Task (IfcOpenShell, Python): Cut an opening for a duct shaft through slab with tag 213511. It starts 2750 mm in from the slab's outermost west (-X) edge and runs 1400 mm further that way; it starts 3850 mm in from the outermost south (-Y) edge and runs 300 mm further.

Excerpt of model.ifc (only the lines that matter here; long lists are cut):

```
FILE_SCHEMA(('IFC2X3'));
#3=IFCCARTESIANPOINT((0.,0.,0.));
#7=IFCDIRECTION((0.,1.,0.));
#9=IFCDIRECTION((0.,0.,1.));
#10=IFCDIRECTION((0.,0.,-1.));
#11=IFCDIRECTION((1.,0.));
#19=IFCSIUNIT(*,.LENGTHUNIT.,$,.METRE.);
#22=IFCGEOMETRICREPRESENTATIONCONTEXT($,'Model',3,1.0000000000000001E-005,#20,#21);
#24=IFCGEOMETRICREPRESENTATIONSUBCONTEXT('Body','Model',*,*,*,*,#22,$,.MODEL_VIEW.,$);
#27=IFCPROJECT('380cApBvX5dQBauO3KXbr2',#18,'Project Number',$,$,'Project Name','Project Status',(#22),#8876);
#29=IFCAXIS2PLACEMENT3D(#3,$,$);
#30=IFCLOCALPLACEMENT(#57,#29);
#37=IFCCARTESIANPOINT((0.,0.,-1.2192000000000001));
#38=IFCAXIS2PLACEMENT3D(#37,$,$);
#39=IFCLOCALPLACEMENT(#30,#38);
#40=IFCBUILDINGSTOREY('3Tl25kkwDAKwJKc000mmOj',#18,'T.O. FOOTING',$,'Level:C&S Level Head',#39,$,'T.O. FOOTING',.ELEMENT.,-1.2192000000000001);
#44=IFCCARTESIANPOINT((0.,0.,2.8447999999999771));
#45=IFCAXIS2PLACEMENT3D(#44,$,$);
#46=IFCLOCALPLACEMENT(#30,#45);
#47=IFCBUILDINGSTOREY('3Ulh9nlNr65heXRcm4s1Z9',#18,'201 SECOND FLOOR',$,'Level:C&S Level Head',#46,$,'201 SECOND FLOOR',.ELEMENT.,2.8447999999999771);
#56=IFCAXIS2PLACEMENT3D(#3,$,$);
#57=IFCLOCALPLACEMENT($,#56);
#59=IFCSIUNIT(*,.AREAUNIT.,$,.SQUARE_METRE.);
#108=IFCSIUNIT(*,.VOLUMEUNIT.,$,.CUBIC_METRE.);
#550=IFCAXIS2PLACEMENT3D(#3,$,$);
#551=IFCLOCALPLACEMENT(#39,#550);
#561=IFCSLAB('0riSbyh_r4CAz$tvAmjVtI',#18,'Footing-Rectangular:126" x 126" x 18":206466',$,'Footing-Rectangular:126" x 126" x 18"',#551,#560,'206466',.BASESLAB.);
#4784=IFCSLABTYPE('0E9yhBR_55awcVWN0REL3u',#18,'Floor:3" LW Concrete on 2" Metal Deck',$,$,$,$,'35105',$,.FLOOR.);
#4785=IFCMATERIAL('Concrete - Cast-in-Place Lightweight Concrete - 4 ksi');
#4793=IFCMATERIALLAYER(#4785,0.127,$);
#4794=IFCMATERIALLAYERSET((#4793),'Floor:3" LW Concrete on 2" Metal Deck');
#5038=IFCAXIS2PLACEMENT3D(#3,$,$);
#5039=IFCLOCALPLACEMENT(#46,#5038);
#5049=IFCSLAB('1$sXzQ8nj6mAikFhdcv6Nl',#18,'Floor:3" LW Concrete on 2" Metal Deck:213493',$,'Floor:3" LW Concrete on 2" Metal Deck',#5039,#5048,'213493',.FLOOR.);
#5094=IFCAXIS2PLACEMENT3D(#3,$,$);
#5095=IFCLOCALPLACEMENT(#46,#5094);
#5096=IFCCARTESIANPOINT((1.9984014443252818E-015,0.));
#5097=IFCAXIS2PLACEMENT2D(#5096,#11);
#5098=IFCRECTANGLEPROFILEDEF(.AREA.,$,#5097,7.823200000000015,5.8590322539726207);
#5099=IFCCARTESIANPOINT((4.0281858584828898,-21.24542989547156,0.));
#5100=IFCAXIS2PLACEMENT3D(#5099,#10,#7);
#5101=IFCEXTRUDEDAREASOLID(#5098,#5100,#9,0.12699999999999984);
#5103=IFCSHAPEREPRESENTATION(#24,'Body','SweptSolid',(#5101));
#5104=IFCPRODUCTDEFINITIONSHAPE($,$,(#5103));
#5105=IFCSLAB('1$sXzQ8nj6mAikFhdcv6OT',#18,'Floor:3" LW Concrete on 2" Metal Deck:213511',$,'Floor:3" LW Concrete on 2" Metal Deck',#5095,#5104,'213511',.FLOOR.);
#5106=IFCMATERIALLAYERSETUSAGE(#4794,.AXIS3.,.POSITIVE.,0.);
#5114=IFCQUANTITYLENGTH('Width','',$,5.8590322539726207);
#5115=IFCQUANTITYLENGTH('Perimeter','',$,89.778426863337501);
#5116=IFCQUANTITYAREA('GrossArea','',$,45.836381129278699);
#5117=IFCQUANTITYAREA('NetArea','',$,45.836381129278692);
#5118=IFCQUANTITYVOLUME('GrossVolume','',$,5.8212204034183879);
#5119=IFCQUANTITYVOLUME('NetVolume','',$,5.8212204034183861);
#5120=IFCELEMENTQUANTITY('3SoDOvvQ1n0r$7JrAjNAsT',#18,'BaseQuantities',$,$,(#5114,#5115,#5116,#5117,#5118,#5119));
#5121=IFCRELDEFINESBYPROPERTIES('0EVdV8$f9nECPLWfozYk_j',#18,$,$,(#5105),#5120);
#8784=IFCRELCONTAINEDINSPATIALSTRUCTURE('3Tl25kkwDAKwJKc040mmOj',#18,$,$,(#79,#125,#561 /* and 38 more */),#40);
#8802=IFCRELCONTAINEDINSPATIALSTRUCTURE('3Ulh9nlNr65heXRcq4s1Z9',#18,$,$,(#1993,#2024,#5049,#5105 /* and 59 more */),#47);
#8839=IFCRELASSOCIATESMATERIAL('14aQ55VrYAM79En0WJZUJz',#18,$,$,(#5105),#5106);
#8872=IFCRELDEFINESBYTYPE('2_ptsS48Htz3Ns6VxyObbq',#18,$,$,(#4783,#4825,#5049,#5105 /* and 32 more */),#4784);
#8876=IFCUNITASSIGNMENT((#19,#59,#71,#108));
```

```python
import numpy as np
import ifcopenshell
import ifcopenshell.api.feature
import ifcopenshell.api.geometry
import ifcopenshell.api.pset
import ifcopenshell.api.root
import ifcopenshell.geom
import ifcopenshell.util.element
import ifcopenshell.util.placement
import ifcopenshell.util.representation
import ifcopenshell.util.shape
import ifcopenshell.util.unit

model = ifcopenshell.open("model.ifc")
unit_scale = ifcopenshell.util.unit.calculate_unit_scale(model)
area_scale = ifcopenshell.util.unit.calculate_unit_scale(model, "AREAUNIT")
volume_scale = ifcopenshell.util.unit.calculate_unit_scale(model, "VOLUMEUNIT")
settings = ifcopenshell.geom.settings()


def volume(element):
    """Net volume in cubic metres, openings subtracted."""
    shape = ifcopenshell.geom.create_shape(settings, element)
    return ifcopenshell.util.shape.get_volume(shape.geometry)


slab = model.by_guid("1$sXzQ8nj6mAikFhdcv6OT")
before = volume(slab)

# Extent in the slab's own axes, in metres. The edges named are its -X and -Y sides.
slab_shape = ifcopenshell.geom.create_shape(settings, slab)
vertices = ifcopenshell.util.shape.get_vertices(slab_shape.geometry)
x_min, y_min, bottom = vertices.min(axis=0)
top = vertices[:, 2].max()

opening = ifcopenshell.api.root.create_entity(model, ifc_class="IfcOpeningElement", name="Duct shaft opening")
context = ifcopenshell.util.representation.get_context(model, "Model", "Body", "MODEL_VIEW")
width, depth = 1.4, 0.3
outline = [(0.0, 0.0), (width, 0.0), (width, depth), (0.0, depth), (0.0, 0.0)]
# Overshoot both faces by 50 mm so the cut is clean.
shape = ifcopenshell.api.geometry.add_slab_representation(
    model, context=context, depth=top - bottom + 0.1, polyline=outline
)
ifcopenshell.api.geometry.assign_representation(model, product=opening, representation=shape)

matrix = ifcopenshell.util.placement.get_local_placement(slab.ObjectPlacement)
matrix[:, 3] = matrix @ np.append(np.array([x_min + 2.75, y_min + 3.85, bottom - 0.05]) / unit_scale, 1.0)
ifcopenshell.api.geometry.edit_object_placement(model, product=opening, matrix=matrix, is_si=False)
ifcopenshell.api.feature.add_feature(model, feature=opening, element=slab)

after = volume(slab)

# Update the slab's stored quantities.
qto = model.by_id(ifcopenshell.util.element.get_pset(slab, "BaseQuantities", should_inherit=False)["id"])
ifcopenshell.api.pset.edit_qto(model, qto=qto, properties={
    "NetArea": after / (top - bottom) / area_scale,
    "NetVolume": after / volume_scale,
})

print(f"slab volume {before:.3f} -> {after:.3f} m3")

model.write("model_updated.ifc")
```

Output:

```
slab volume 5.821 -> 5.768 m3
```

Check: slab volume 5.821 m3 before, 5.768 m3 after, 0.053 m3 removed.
